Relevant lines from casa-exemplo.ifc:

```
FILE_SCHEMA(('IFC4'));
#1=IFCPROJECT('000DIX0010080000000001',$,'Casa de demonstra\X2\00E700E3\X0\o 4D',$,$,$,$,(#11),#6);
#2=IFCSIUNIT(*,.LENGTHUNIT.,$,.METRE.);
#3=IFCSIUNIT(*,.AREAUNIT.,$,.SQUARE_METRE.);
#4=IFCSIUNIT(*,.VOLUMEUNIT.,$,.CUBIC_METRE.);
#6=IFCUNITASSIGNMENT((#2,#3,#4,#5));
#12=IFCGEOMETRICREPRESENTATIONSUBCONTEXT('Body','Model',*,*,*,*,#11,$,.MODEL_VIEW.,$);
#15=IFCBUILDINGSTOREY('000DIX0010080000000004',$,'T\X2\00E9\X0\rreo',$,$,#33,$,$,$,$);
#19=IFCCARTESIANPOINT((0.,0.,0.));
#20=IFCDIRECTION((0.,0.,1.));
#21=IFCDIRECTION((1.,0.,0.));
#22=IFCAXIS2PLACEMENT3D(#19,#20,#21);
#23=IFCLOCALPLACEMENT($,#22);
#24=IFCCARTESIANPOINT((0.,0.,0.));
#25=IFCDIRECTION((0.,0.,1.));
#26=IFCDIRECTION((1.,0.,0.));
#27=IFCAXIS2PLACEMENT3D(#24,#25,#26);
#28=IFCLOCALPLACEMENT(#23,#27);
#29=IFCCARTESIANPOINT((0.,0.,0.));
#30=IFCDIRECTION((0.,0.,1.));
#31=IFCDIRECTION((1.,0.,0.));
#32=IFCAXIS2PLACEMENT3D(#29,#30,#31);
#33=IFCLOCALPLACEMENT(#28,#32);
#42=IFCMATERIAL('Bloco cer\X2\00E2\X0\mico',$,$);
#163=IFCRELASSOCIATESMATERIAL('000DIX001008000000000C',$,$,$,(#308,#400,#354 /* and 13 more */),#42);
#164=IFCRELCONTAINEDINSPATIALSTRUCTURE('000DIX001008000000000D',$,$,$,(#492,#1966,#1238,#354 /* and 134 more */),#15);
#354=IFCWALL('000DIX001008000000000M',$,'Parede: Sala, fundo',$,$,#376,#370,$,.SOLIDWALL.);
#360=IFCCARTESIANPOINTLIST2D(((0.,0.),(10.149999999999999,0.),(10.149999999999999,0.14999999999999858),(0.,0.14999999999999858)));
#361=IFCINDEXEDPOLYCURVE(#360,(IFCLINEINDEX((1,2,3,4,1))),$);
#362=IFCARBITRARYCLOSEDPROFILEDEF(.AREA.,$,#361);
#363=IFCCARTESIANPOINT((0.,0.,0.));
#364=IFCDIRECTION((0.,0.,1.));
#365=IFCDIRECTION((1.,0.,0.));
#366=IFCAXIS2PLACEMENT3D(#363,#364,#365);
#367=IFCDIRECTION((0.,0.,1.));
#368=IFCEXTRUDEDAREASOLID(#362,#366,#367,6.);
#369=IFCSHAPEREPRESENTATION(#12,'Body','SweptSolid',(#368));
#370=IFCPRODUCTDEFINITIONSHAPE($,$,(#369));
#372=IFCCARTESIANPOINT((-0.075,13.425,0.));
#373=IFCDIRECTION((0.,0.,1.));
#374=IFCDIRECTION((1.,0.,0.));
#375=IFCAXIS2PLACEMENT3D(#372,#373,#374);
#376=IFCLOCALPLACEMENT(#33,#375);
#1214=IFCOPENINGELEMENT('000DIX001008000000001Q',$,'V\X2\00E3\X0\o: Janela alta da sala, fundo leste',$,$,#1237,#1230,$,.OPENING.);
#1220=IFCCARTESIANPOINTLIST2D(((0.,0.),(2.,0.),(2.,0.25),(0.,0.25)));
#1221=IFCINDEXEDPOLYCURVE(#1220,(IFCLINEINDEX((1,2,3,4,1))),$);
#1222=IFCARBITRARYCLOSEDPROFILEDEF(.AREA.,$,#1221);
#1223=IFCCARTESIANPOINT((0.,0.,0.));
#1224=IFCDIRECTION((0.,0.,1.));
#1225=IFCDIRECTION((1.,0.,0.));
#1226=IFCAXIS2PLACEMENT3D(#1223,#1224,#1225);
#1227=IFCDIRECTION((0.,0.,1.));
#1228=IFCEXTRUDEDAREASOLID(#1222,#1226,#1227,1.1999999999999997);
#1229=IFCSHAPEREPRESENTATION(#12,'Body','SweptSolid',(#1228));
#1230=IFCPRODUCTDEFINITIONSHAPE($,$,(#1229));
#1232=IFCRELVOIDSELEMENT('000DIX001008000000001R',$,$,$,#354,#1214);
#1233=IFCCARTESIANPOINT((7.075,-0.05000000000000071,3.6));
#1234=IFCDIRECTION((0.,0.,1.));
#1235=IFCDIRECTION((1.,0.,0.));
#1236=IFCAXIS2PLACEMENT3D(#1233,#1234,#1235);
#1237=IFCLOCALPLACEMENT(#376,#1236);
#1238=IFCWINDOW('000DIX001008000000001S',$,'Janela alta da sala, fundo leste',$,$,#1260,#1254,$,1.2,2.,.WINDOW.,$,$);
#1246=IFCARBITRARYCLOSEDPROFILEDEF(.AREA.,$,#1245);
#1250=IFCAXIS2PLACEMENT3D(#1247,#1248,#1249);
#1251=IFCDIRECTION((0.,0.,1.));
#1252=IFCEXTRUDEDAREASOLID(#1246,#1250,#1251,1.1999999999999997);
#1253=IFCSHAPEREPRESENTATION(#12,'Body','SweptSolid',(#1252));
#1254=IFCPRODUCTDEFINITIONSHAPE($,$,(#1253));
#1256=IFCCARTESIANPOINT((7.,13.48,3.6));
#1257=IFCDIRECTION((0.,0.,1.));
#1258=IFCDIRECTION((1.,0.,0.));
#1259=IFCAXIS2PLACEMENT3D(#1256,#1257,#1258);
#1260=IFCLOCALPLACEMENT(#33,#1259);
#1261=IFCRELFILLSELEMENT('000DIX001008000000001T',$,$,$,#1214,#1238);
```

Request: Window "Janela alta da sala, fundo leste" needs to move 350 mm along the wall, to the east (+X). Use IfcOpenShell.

```python
import ifcopenshell
import ifcopenshell.api.geometry
import ifcopenshell.util.placement

model = ifcopenshell.open("casa-exemplo.ifc")

window = model.by_guid("000DIX001008000000001S")
opening = window.FillsVoids[0].RelatingOpeningElement
wall = opening.VoidsElements[0].RelatingBuildingElement

wall_matrix = ifcopenshell.util.placement.get_local_placement(wall.ObjectPlacement)
shift = wall_matrix[:3, 0] * 0.35
before = ifcopenshell.util.placement.get_local_placement(window.ObjectPlacement)[:3, 3].copy()

# The window is not placed relative to its opening, so move both.
for product in (opening, window):
    matrix = ifcopenshell.util.placement.get_local_placement(product.ObjectPlacement)
    matrix[:3, 3] += shift
    ifcopenshell.api.geometry.edit_object_placement(model, product=product, matrix=matrix, is_si=False)

after = ifcopenshell.util.placement.get_local_placement(window.ObjectPlacement)[:3, 3]
print("window moved by", (after - before).round(3) + 0.0)

model.write("casa-exemplo_updated.ifc")
```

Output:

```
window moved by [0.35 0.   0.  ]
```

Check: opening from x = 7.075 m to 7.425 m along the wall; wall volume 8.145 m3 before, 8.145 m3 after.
